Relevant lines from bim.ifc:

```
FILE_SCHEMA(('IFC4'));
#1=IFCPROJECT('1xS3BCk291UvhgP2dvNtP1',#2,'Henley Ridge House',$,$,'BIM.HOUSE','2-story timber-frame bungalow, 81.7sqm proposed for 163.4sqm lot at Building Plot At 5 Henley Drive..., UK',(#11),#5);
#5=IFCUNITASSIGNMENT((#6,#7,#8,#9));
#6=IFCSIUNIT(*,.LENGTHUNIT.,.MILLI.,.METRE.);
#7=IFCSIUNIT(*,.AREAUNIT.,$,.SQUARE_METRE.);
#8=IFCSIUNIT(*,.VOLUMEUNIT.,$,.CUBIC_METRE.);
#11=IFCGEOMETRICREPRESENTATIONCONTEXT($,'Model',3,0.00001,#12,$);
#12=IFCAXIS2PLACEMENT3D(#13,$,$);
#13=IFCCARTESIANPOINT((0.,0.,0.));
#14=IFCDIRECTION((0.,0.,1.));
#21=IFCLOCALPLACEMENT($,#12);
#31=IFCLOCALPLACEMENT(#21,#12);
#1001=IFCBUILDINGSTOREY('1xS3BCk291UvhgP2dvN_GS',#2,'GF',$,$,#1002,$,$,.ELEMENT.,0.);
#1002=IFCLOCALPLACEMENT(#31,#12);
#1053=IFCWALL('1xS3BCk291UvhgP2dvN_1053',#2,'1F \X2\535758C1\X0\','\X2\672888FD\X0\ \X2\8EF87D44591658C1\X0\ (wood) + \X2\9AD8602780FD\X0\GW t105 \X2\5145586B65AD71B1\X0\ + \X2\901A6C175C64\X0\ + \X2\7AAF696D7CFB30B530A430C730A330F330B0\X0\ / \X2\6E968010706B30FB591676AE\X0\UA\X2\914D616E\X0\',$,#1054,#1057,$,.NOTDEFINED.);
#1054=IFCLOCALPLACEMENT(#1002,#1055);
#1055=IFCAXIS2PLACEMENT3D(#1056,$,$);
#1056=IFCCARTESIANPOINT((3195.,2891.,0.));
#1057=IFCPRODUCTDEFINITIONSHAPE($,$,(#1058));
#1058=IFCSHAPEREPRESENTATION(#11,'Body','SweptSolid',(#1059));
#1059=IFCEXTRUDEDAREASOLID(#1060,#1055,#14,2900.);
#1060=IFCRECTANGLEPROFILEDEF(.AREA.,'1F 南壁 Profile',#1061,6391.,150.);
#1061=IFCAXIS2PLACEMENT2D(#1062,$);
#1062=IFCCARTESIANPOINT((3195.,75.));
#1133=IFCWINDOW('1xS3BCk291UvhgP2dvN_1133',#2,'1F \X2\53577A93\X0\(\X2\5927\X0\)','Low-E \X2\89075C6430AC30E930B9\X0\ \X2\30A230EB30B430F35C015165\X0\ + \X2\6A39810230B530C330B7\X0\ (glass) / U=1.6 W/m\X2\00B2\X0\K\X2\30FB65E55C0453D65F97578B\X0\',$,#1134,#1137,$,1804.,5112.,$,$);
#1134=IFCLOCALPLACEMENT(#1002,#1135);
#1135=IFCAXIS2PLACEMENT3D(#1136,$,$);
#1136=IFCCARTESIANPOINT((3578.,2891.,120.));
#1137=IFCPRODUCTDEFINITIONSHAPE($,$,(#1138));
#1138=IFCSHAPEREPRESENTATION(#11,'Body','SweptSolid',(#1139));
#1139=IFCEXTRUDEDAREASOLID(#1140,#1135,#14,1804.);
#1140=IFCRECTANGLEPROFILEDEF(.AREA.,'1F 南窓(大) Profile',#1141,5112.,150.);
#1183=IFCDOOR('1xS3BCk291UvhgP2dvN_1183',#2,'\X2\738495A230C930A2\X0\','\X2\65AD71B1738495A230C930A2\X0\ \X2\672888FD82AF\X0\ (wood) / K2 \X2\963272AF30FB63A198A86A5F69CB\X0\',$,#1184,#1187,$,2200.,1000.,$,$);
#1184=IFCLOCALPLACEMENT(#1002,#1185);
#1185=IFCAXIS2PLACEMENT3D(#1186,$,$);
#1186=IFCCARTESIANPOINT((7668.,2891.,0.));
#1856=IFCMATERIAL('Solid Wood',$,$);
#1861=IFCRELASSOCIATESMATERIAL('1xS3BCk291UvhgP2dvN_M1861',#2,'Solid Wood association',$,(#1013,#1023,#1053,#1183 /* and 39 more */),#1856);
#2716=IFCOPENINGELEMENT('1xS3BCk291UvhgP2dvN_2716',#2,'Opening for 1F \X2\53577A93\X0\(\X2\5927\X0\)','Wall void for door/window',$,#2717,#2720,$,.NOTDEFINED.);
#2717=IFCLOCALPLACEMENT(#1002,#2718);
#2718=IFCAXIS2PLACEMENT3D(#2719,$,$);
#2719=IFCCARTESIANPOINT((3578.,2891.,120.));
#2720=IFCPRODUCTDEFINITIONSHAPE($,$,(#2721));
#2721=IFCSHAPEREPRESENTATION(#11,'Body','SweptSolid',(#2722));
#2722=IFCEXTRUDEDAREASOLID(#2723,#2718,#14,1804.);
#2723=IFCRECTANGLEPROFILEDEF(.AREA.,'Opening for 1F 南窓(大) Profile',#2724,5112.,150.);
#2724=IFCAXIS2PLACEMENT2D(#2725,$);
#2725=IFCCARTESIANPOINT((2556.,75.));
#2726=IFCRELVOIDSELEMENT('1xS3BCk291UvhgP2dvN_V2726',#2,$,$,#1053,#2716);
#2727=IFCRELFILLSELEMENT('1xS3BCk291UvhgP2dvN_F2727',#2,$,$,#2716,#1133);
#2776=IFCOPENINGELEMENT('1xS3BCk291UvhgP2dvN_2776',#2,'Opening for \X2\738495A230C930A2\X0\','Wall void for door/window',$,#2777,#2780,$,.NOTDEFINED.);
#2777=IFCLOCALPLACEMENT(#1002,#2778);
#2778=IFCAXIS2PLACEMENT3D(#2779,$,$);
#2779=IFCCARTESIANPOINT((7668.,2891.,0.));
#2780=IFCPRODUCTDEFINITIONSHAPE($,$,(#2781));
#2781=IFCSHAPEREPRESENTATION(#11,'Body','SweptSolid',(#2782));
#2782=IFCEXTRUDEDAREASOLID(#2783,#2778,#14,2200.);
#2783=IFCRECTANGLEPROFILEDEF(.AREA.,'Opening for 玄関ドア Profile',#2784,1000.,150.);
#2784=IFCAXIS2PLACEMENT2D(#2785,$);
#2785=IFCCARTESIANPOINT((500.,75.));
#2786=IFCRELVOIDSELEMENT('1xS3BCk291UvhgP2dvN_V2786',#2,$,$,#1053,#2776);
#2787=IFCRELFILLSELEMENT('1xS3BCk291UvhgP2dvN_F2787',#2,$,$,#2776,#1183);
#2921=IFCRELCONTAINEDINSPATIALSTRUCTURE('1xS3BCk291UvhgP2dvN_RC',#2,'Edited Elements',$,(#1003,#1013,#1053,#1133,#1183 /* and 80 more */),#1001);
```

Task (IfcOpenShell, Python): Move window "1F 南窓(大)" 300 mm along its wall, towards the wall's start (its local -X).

```python
import ifcopenshell
import ifcopenshell.api.geometry
import ifcopenshell.util.placement
import ifcopenshell.util.unit

model = ifcopenshell.open("bim.ifc")
unit_scale = ifcopenshell.util.unit.calculate_unit_scale(model)

window = model.by_guid("1xS3BCk291UvhgP2dvN_1133")
opening = window.FillsVoids[0].RelatingOpeningElement
wall = opening.VoidsElements[0].RelatingBuildingElement

wall_matrix = ifcopenshell.util.placement.get_local_placement(wall.ObjectPlacement)
shift = wall_matrix[:3, 0] * -0.3 / unit_scale
before = ifcopenshell.util.placement.get_local_placement(window.ObjectPlacement)[:3, 3].copy()

# The window is not placed relative to its opening, so move both.
for product in (opening, window):
    matrix = ifcopenshell.util.placement.get_local_placement(product.ObjectPlacement)
    matrix[:3, 3] += shift
    ifcopenshell.api.geometry.edit_object_placement(model, product=product, matrix=matrix, is_si=False)

after = ifcopenshell.util.placement.get_local_placement(window.ObjectPlacement)[:3, 3]
print("window moved by", (after - before).round(3) + 0.0)

model.write("bim_updated.ifc")
```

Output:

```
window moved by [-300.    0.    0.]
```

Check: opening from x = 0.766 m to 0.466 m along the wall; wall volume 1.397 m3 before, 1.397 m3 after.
